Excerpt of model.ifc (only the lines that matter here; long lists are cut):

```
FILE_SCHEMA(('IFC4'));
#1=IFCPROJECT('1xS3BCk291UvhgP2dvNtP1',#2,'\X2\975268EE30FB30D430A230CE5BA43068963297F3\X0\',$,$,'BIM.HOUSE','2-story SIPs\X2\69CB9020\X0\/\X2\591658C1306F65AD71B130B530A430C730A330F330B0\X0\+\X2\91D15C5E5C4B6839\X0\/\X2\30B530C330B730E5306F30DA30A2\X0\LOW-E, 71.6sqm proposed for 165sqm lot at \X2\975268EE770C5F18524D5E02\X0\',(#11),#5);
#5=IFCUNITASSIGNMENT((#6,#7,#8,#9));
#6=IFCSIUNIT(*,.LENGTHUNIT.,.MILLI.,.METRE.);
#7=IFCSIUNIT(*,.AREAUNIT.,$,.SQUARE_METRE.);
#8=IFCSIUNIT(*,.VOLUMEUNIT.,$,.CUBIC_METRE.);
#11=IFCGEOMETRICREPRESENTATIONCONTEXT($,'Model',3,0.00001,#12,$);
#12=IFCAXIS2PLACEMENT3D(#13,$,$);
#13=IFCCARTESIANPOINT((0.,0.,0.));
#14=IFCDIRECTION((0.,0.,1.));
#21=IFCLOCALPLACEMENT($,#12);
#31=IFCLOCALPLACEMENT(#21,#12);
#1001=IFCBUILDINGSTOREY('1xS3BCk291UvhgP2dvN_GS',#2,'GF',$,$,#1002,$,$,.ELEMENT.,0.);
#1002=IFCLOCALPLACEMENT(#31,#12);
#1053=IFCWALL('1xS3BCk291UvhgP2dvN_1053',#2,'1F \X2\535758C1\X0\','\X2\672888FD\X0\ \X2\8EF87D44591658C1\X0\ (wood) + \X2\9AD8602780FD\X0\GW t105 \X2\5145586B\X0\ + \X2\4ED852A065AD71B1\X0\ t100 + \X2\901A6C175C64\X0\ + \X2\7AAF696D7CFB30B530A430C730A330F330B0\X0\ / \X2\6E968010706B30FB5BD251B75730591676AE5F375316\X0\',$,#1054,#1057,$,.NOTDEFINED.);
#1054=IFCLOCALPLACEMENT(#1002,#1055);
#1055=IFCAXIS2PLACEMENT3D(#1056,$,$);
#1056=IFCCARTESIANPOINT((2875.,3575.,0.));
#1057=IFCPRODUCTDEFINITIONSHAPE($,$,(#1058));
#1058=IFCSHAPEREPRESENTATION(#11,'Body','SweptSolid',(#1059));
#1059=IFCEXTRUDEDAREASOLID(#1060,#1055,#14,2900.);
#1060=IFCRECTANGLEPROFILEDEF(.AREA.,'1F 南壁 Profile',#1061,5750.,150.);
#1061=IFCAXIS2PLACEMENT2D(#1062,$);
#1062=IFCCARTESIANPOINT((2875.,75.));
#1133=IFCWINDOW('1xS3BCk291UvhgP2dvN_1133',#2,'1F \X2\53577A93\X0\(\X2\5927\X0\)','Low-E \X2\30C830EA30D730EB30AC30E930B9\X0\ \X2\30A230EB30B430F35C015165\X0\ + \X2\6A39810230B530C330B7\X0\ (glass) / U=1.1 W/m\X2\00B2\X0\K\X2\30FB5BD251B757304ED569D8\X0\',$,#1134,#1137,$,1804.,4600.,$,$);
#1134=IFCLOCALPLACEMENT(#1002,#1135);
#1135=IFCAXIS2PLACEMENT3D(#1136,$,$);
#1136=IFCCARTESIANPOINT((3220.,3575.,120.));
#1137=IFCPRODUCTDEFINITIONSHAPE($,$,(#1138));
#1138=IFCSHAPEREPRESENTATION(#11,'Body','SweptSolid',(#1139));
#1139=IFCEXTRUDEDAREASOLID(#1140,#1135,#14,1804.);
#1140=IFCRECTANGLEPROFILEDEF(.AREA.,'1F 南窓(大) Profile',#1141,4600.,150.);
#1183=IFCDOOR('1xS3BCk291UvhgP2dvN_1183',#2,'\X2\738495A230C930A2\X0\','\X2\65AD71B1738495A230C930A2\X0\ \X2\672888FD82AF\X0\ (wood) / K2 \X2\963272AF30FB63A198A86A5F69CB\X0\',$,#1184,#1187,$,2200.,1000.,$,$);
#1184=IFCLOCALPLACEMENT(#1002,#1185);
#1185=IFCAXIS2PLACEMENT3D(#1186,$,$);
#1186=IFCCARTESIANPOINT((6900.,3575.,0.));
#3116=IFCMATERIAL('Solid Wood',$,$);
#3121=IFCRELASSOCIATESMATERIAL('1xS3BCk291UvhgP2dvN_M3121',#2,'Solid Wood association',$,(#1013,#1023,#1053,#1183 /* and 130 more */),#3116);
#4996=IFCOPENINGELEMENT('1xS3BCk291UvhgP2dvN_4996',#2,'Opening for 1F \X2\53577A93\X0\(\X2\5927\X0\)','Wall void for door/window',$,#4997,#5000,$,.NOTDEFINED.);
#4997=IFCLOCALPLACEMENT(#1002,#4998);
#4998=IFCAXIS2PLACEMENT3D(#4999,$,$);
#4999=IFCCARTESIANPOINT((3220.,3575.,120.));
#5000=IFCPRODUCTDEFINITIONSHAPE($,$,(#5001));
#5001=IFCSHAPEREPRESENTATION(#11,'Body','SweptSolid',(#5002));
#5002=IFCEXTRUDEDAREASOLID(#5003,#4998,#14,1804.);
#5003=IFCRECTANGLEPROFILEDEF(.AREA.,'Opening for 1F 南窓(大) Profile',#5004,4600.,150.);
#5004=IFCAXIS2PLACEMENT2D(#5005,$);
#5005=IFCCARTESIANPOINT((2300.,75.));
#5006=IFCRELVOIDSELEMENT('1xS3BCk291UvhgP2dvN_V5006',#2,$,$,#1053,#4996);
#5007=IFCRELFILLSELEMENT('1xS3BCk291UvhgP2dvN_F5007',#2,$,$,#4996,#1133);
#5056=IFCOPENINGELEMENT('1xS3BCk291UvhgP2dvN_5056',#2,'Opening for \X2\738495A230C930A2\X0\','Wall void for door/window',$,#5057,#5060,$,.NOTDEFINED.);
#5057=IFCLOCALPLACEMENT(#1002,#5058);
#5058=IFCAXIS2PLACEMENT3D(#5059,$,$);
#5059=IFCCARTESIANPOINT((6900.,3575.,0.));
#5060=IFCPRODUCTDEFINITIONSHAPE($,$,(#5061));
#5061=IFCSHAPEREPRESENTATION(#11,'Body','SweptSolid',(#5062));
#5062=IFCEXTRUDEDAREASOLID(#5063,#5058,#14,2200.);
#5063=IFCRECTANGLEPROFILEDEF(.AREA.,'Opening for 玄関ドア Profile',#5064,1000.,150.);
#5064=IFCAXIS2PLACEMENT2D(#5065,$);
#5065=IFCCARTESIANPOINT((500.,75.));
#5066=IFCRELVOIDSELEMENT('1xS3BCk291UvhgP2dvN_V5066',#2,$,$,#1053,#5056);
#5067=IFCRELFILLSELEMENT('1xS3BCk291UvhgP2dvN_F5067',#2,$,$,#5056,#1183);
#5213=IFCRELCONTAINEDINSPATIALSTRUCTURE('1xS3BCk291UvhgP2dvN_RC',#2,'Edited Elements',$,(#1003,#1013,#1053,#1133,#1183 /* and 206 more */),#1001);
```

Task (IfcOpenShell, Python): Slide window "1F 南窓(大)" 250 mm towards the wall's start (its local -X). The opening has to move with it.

```python
import ifcopenshell
import ifcopenshell.api.geometry
import ifcopenshell.util.placement
import ifcopenshell.util.unit

model = ifcopenshell.open("model.ifc")
unit_scale = ifcopenshell.util.unit.calculate_unit_scale(model)

window = model.by_guid("1xS3BCk291UvhgP2dvN_1133")
opening = window.FillsVoids[0].RelatingOpeningElement
wall = opening.VoidsElements[0].RelatingBuildingElement

wall_matrix = ifcopenshell.util.placement.get_local_placement(wall.ObjectPlacement)
shift = wall_matrix[:3, 0] * -0.25 / unit_scale
before = ifcopenshell.util.placement.get_local_placement(window.ObjectPlacement)[:3, 3].copy()

# The window is not placed relative to its opening, so move both.
for product in (opening, window):
    matrix = ifcopenshell.util.placement.get_local_placement(product.ObjectPlacement)
    matrix[:3, 3] += shift
    ifcopenshell.api.geometry.edit_object_placement(model, product=product, matrix=matrix, is_si=False)

after = ifcopenshell.util.placement.get_local_placement(window.ObjectPlacement)[:3, 3]
print("window moved by", (after - before).round(3) + 0.0)

model.write("model-out.ifc")
```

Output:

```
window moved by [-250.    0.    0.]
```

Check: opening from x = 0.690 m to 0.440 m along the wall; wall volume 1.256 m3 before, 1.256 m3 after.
